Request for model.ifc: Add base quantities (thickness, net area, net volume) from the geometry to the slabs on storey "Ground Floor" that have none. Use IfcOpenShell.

First a look at what the model holds.

```python
import ifcopenshell
import ifcopenshell.util.element
import ifcopenshell.util.unit

model = ifcopenshell.open("model.ifc")
print(model.schema)
for unit_type in ("LENGTHUNIT", "AREAUNIT", "VOLUMEUNIT"):
    print(unit_type, ifcopenshell.util.unit.calculate_unit_scale(model, unit_type))
storey = next(s for s in model.by_type("IfcBuildingStorey") if s.Name == "Ground Floor")
slabs = [e for e in ifcopenshell.util.element.get_decomposition(storey) if e.is_a("IfcSlab")]
for e in sorted(slabs, key=lambda e: e.id()):
    print(e.id(), e.is_a(), e.Name, list(ifcopenshell.util.element.get_psets(e, qtos_only=True)), sep=" | ")
```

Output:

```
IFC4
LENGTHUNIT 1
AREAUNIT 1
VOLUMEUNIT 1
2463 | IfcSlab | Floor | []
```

```python
import ifcopenshell
import ifcopenshell.api.pset
import ifcopenshell.geom
import ifcopenshell.util.element
import ifcopenshell.util.shape
import ifcopenshell.util.unit

model = ifcopenshell.open("model.ifc")
unit_scale = ifcopenshell.util.unit.calculate_unit_scale(model)
area_scale = ifcopenshell.util.unit.calculate_unit_scale(model, "AREAUNIT")
volume_scale = ifcopenshell.util.unit.calculate_unit_scale(model, "VOLUMEUNIT")
settings = ifcopenshell.geom.settings()

storey = next(s for s in model.by_type("IfcBuildingStorey") if s.Name == "Ground Floor")
slabs = [e for e in ifcopenshell.util.element.get_decomposition(storey) if e.is_a("IfcSlab")]

for e in sorted(slabs, key=lambda e: e.id()):
    if ifcopenshell.util.element.get_psets(e, qtos_only=True, should_inherit=False):
        continue
    # Geometry comes back in metres, in the element's own axes.
    shape = ifcopenshell.geom.create_shape(settings, e)
    values = {
        "Width": ifcopenshell.util.shape.get_z(shape.geometry) / unit_scale,
        "NetArea": ifcopenshell.util.shape.get_footprint_area(shape.geometry) / area_scale,
        "NetVolume": ifcopenshell.util.shape.get_volume(shape.geometry) / volume_scale,
    }
    qto = ifcopenshell.api.pset.add_qto(model, product=e, name="Qto_SlabBaseQuantities")
    ifcopenshell.api.pset.edit_qto(model, qto=qto, properties=values)
    print(e.id(), {k: round(v, 3) for k, v in values.items()})

model.write("model_v2.ifc")
```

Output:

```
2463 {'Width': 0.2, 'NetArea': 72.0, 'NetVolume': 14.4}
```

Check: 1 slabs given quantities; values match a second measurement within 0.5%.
